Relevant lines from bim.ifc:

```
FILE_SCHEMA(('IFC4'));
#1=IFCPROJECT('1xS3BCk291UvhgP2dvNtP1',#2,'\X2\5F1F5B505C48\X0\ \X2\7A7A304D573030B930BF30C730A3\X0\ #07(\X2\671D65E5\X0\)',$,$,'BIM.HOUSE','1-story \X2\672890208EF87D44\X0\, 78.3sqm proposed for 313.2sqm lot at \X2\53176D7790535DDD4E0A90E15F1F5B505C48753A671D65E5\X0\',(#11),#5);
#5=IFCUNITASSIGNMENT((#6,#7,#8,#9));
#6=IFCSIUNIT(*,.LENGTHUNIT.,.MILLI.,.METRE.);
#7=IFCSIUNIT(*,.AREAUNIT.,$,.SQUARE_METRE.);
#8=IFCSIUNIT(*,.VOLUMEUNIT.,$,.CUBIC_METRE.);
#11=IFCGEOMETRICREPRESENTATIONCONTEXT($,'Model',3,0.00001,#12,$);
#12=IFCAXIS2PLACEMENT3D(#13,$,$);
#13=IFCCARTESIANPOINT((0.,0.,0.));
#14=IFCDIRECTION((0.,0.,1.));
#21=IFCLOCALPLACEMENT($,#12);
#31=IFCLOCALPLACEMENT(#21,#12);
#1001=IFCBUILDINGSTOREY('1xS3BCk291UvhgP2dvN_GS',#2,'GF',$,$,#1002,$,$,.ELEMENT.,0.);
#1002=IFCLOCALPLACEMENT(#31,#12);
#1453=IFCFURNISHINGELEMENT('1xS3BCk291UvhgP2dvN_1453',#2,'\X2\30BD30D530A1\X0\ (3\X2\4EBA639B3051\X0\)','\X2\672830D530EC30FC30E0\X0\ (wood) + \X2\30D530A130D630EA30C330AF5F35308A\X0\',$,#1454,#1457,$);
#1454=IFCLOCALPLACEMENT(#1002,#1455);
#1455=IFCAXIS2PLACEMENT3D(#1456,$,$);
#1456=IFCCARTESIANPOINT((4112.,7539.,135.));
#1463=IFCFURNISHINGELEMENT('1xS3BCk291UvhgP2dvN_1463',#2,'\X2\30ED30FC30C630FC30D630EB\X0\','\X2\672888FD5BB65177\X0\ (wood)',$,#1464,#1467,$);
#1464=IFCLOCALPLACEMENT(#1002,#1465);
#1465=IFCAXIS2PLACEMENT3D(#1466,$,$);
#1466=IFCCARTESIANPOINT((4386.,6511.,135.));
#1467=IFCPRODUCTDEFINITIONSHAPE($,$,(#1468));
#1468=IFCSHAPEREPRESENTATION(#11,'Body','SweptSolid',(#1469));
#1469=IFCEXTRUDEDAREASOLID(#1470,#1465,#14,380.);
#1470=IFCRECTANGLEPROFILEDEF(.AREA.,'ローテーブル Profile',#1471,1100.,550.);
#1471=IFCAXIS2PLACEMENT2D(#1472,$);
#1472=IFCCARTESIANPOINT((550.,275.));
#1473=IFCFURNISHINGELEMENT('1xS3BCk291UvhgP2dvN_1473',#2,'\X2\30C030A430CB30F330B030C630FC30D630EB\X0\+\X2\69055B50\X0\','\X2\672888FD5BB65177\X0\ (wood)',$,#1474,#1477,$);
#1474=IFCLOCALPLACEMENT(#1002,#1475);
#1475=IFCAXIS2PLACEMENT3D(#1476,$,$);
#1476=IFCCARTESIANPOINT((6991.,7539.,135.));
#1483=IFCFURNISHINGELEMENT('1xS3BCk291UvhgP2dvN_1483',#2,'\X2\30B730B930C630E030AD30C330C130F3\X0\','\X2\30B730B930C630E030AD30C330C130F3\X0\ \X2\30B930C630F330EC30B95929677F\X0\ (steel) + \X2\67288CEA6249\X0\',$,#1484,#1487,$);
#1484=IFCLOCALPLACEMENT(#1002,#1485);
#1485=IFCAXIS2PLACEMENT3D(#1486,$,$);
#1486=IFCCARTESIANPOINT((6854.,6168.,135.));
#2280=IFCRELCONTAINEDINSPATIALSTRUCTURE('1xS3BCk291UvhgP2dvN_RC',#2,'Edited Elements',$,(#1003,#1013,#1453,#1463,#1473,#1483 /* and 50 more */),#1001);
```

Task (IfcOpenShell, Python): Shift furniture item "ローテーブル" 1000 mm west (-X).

```python
import ifcopenshell
import ifcopenshell.api.geometry
import ifcopenshell.util.placement
import ifcopenshell.util.unit

model = ifcopenshell.open("bim.ifc")
unit_scale = ifcopenshell.util.unit.calculate_unit_scale(model)

item = model.by_id(1463)
matrix = ifcopenshell.util.placement.get_local_placement(item.ObjectPlacement)
matrix[0, 3] -= 1 / unit_scale
ifcopenshell.api.geometry.edit_object_placement(model, product=item, matrix=matrix, is_si=False)

print(ifcopenshell.util.placement.get_local_placement(item.ObjectPlacement).round(3) + 0.0)

model.write("bim-out.ifc")
```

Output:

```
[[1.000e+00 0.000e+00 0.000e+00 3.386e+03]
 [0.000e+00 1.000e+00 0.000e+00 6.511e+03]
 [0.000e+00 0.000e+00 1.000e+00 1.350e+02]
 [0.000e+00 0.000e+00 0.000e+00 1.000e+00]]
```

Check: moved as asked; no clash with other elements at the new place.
